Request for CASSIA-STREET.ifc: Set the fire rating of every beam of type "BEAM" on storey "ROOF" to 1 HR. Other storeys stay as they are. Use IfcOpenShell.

First a look at what the model holds.

```python
import ifcopenshell
import ifcopenshell.util.element

model = ifcopenshell.open("CASSIA-STREET.ifc")
print(model.schema)
storey = next(s for s in model.by_type("IfcBuildingStorey") if s.Name == "ROOF")
beams = [e for e in ifcopenshell.util.element.get_decomposition(storey) if e.is_a("IfcBeam")]
seen = {}
for e in beams:
    element_type = ifcopenshell.util.element.get_type(e)
    key = (element_type.Name if element_type != e and element_type else None, ifcopenshell.util.element.get_pset(e, "Pset_BeamCommon", "FireRating"))
    seen[key] = seen.get(key, 0) + 1
for (name, value), count in sorted(seen.items(), key=str):
    print(count, "x", name, "|", value)
```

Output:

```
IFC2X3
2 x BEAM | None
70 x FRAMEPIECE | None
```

```python
import ifcopenshell
import ifcopenshell.api.pset
import ifcopenshell.util.element

model = ifcopenshell.open("CASSIA-STREET.ifc")

storey = next(s for s in model.by_type("IfcBuildingStorey") if s.Name == "ROOF")
beams = [e for e in ifcopenshell.util.element.get_decomposition(storey) if e.is_a("IfcBeam")]

count = 0
for e in beams:
    element_type = ifcopenshell.util.element.get_type(e)
    if element_type in (None, e) or element_type.Name != "BEAM":
        continue
    # add_pset returns the element's existing set when there is one.
    pset = ifcopenshell.api.pset.add_pset(model, product=e, name="Pset_BeamCommon")
    ifcopenshell.api.pset.edit_pset(model, pset=pset, properties={"FireRating": "1 HR"})
    count += 1

print(count, "beams updated")

model.write("CASSIA-STREET_updated.ifc")
```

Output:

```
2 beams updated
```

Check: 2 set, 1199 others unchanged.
